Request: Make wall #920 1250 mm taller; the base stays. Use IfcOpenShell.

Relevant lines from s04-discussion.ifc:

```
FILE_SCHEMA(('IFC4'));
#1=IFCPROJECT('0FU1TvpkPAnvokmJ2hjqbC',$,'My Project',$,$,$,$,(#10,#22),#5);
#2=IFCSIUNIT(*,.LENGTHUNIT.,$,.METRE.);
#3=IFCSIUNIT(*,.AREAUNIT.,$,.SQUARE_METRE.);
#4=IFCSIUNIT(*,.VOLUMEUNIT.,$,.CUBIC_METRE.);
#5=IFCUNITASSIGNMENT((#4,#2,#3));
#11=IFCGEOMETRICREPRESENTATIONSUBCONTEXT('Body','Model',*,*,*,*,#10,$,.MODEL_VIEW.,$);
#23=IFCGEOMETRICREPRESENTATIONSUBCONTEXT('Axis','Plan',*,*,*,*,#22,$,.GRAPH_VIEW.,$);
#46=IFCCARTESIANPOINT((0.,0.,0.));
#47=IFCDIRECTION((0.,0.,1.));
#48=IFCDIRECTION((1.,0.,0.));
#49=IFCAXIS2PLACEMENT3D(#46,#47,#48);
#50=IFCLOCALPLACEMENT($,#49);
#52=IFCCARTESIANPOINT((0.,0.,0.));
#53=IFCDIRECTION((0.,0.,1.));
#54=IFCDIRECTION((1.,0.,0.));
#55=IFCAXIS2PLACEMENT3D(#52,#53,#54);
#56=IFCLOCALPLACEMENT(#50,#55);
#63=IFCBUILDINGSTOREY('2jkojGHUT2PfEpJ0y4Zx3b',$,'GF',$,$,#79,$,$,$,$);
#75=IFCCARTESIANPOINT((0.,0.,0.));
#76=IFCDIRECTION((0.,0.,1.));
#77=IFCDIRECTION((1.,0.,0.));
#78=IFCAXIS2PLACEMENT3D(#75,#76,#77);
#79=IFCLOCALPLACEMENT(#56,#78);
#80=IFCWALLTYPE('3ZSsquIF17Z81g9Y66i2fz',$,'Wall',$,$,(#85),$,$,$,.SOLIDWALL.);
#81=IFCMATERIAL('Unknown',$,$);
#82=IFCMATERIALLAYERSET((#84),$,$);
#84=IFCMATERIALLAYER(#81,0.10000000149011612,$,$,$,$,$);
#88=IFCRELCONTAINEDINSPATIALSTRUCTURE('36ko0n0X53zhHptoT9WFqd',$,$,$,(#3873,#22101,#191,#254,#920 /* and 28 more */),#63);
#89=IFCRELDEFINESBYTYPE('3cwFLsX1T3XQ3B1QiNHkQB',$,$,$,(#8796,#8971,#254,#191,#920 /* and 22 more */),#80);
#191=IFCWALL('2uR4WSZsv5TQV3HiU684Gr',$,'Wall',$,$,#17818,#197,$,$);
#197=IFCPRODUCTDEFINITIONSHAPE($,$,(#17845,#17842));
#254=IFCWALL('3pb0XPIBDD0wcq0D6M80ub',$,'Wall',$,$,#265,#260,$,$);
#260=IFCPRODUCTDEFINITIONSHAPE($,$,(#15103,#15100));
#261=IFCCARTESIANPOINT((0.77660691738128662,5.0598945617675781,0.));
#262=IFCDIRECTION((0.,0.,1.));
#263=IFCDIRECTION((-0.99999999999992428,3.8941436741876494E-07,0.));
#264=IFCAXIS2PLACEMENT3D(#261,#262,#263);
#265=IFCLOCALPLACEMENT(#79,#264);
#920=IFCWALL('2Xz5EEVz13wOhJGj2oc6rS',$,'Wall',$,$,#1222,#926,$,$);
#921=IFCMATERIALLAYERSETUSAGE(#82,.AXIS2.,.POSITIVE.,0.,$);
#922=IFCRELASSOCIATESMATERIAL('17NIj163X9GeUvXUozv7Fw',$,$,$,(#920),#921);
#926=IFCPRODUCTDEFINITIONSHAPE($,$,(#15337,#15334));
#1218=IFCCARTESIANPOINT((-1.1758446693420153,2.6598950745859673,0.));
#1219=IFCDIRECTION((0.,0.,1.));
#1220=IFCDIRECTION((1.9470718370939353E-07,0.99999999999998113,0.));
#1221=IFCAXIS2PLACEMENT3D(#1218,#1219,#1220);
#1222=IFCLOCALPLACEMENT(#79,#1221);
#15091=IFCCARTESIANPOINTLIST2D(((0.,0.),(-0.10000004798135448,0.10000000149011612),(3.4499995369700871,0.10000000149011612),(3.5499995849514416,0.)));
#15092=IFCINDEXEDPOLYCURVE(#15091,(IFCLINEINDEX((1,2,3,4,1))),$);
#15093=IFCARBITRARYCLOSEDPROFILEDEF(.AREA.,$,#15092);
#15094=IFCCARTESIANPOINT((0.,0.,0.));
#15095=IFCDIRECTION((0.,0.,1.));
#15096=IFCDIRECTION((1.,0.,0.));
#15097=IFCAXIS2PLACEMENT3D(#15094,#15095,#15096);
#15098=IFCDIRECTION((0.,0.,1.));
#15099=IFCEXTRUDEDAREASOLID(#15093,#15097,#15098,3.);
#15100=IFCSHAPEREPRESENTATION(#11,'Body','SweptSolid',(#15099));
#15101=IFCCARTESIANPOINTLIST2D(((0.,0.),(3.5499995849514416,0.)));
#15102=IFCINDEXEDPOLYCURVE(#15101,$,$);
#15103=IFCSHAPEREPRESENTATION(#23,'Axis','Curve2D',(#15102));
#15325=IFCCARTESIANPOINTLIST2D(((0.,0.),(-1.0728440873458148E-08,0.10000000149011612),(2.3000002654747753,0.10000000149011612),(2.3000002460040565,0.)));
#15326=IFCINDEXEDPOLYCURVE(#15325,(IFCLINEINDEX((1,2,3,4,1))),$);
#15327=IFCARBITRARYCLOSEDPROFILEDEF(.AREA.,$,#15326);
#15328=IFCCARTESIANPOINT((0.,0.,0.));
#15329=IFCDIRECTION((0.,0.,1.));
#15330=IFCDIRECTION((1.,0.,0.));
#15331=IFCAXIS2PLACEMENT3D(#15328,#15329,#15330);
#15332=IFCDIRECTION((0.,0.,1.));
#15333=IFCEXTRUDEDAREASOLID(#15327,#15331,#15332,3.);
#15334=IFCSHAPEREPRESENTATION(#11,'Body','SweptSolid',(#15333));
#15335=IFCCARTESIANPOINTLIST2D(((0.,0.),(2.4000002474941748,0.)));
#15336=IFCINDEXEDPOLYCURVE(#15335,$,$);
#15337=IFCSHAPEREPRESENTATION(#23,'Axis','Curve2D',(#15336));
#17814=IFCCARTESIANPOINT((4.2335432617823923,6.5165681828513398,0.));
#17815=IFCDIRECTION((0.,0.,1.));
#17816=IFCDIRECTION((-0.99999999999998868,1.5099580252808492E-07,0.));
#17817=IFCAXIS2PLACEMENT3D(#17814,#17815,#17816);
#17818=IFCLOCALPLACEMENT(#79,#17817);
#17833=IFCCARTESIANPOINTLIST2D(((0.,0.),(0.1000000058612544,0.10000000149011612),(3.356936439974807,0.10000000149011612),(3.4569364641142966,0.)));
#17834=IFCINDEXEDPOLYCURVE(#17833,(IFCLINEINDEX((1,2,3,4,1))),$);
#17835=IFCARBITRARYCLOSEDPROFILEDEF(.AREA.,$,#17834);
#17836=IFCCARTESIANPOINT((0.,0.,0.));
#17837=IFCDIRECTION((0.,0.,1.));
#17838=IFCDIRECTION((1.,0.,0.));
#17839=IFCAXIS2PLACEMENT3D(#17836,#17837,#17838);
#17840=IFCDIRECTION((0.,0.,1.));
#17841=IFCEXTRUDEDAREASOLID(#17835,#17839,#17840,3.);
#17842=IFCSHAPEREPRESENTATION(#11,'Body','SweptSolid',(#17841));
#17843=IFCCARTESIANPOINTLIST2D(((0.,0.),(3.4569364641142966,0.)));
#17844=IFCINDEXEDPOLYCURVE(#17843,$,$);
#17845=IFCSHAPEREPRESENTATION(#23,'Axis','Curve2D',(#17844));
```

```python
import ifcopenshell
import ifcopenshell.geom
import ifcopenshell.util.representation
import ifcopenshell.util.shape
import ifcopenshell.util.unit

model = ifcopenshell.open("s04-discussion.ifc")
unit_scale = ifcopenshell.util.unit.calculate_unit_scale(model)
settings = ifcopenshell.geom.settings()


def volume(element):
    """Net volume in cubic metres, openings subtracted."""
    shape = ifcopenshell.geom.create_shape(settings, element)
    return ifcopenshell.util.shape.get_volume(shape.geometry)


wall = model.by_guid("2Xz5EEVz13wOhJGj2oc6rS")
before = volume(wall)

body = ifcopenshell.util.representation.get_representation(wall, "Model", "Body")
solid = body.Items[0]
old_height = solid.Depth
solid.Depth += 1.25 / unit_scale
after = volume(wall)

print(f"height {old_height:g} -> {solid.Depth:g}, volume {before:.3f} -> {after:.3f} m3")

model.write("s04-discussion_rev.ifc")
```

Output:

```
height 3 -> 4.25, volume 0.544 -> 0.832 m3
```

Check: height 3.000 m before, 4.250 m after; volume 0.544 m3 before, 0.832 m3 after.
